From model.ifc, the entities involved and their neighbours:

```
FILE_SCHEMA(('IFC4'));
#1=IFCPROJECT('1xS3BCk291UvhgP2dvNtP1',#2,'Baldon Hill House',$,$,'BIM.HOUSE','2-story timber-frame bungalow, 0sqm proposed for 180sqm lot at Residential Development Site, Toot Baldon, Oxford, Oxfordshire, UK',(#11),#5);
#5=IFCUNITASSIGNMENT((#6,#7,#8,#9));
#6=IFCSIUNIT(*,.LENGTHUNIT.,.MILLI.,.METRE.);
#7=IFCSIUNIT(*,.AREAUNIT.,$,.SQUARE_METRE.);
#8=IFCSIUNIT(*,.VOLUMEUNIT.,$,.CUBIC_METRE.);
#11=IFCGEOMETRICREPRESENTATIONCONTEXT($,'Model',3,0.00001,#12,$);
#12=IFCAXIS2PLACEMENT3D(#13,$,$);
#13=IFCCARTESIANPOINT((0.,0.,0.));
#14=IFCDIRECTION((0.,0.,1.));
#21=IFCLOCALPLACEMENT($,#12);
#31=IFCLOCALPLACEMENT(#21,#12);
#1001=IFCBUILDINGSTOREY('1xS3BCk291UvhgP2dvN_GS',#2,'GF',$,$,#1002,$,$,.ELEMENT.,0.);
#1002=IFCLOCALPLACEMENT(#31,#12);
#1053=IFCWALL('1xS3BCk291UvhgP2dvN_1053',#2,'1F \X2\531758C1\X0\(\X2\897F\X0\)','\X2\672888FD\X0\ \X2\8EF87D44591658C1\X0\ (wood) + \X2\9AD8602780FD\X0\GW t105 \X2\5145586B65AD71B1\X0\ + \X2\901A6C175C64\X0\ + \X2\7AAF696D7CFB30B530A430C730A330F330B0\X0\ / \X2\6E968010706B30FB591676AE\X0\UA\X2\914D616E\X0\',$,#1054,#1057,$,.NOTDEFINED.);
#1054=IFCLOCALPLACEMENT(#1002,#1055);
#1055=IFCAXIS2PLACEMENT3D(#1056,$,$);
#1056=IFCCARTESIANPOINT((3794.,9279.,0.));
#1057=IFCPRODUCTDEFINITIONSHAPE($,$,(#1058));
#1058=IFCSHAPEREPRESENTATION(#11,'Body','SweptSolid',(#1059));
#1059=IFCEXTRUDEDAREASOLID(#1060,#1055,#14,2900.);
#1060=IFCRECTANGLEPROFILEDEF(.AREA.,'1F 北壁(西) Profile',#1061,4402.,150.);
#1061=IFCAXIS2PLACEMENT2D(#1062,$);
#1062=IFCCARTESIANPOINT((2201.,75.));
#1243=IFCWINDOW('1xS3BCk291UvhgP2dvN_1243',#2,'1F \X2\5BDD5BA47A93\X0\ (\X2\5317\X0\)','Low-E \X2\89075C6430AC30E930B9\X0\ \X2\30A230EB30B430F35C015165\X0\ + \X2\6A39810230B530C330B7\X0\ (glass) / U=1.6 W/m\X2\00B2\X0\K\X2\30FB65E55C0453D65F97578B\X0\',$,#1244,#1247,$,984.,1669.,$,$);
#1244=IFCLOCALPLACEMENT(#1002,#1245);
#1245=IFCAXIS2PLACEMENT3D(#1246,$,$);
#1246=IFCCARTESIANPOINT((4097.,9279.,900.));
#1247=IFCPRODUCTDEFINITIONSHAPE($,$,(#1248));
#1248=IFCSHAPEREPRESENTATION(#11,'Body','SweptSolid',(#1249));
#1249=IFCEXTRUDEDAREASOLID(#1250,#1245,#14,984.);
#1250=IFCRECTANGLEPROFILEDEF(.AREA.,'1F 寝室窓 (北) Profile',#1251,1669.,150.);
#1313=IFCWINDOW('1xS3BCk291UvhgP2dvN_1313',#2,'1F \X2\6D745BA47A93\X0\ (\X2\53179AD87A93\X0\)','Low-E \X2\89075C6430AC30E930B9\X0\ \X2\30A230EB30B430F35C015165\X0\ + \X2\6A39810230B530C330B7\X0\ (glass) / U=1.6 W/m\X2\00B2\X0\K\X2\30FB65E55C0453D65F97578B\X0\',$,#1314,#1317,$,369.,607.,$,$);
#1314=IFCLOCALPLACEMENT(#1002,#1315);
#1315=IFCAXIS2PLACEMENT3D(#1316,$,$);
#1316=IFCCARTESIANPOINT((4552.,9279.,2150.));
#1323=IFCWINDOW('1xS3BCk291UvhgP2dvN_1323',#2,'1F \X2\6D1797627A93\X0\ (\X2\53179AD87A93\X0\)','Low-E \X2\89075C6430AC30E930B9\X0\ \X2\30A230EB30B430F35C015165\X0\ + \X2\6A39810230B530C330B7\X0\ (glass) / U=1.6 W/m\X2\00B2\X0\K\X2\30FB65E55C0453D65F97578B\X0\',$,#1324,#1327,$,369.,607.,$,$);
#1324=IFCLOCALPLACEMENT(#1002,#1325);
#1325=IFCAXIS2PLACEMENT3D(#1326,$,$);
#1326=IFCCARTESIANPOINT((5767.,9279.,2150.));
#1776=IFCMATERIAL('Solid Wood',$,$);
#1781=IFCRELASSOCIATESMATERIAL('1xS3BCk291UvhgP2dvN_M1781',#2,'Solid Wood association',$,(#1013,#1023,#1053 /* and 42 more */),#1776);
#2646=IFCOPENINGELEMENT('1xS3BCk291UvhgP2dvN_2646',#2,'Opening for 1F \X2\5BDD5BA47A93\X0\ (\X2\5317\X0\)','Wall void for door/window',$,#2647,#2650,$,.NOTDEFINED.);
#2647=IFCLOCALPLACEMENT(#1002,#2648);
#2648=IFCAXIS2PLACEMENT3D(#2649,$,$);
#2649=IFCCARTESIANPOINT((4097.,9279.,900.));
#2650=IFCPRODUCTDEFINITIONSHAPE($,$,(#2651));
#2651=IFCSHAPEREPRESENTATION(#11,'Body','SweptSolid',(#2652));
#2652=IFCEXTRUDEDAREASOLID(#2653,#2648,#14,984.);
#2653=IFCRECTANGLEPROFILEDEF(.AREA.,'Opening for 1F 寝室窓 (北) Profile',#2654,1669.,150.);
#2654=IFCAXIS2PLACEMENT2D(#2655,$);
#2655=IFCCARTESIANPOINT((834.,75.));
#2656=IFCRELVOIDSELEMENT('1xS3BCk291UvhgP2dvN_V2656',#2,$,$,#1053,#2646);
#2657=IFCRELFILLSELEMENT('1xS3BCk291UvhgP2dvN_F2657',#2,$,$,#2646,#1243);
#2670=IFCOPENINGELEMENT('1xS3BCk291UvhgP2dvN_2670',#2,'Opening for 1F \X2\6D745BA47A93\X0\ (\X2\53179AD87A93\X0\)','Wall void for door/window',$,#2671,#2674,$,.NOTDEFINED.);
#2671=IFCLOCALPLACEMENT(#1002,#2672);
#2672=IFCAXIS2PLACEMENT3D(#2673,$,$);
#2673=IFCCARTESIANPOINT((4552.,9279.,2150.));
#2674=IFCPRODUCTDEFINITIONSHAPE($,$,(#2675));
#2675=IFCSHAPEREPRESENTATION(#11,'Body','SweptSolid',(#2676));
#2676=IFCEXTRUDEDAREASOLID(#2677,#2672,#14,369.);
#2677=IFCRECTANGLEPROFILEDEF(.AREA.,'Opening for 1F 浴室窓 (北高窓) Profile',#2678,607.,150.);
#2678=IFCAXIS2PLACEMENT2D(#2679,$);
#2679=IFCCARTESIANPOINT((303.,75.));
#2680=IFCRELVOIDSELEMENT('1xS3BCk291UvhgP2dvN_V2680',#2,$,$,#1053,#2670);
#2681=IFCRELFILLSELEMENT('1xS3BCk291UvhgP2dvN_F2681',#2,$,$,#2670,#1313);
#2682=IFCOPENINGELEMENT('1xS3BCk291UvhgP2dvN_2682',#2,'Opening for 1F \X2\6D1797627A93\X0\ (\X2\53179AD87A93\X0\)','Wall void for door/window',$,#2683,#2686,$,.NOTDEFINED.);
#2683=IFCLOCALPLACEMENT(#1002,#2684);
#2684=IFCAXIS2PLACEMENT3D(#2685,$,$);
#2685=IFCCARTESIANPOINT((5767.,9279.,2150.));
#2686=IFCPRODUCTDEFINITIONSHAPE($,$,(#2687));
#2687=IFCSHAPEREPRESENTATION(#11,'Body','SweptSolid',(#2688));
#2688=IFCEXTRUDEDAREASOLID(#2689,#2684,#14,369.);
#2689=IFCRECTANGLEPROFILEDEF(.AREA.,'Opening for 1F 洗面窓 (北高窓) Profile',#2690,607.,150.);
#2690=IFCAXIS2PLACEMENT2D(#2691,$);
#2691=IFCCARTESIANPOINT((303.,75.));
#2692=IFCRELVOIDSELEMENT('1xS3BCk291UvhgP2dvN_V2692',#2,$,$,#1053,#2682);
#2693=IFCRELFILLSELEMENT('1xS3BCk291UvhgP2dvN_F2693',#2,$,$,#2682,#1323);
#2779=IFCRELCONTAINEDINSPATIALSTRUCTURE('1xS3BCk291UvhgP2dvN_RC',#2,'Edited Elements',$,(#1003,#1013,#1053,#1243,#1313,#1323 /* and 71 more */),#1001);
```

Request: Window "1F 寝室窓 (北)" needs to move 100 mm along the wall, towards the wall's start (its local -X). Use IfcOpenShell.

```python
import ifcopenshell
import ifcopenshell.api.geometry
import ifcopenshell.util.placement
import ifcopenshell.util.unit

model = ifcopenshell.open("model.ifc")
unit_scale = ifcopenshell.util.unit.calculate_unit_scale(model)

window = model.by_id(1243)
opening = window.FillsVoids[0].RelatingOpeningElement
wall = opening.VoidsElements[0].RelatingBuildingElement

wall_matrix = ifcopenshell.util.placement.get_local_placement(wall.ObjectPlacement)
shift = wall_matrix[:3, 0] * -0.1 / unit_scale
before = ifcopenshell.util.placement.get_local_placement(window.ObjectPlacement)[:3, 3].copy()

# The window is not placed relative to its opening, so move both.
for product in (opening, window):
    matrix = ifcopenshell.util.placement.get_local_placement(product.ObjectPlacement)
    matrix[:3, 3] += shift
    ifcopenshell.api.geometry.edit_object_placement(model, product=product, matrix=matrix, is_si=False)

after = ifcopenshell.util.placement.get_local_placement(window.ObjectPlacement)[:3, 3]
print("window moved by", (after - before).round(3) + 0.0)

model.write("model_updated.ifc")
```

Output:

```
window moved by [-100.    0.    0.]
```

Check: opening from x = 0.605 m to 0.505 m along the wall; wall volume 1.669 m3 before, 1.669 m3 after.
